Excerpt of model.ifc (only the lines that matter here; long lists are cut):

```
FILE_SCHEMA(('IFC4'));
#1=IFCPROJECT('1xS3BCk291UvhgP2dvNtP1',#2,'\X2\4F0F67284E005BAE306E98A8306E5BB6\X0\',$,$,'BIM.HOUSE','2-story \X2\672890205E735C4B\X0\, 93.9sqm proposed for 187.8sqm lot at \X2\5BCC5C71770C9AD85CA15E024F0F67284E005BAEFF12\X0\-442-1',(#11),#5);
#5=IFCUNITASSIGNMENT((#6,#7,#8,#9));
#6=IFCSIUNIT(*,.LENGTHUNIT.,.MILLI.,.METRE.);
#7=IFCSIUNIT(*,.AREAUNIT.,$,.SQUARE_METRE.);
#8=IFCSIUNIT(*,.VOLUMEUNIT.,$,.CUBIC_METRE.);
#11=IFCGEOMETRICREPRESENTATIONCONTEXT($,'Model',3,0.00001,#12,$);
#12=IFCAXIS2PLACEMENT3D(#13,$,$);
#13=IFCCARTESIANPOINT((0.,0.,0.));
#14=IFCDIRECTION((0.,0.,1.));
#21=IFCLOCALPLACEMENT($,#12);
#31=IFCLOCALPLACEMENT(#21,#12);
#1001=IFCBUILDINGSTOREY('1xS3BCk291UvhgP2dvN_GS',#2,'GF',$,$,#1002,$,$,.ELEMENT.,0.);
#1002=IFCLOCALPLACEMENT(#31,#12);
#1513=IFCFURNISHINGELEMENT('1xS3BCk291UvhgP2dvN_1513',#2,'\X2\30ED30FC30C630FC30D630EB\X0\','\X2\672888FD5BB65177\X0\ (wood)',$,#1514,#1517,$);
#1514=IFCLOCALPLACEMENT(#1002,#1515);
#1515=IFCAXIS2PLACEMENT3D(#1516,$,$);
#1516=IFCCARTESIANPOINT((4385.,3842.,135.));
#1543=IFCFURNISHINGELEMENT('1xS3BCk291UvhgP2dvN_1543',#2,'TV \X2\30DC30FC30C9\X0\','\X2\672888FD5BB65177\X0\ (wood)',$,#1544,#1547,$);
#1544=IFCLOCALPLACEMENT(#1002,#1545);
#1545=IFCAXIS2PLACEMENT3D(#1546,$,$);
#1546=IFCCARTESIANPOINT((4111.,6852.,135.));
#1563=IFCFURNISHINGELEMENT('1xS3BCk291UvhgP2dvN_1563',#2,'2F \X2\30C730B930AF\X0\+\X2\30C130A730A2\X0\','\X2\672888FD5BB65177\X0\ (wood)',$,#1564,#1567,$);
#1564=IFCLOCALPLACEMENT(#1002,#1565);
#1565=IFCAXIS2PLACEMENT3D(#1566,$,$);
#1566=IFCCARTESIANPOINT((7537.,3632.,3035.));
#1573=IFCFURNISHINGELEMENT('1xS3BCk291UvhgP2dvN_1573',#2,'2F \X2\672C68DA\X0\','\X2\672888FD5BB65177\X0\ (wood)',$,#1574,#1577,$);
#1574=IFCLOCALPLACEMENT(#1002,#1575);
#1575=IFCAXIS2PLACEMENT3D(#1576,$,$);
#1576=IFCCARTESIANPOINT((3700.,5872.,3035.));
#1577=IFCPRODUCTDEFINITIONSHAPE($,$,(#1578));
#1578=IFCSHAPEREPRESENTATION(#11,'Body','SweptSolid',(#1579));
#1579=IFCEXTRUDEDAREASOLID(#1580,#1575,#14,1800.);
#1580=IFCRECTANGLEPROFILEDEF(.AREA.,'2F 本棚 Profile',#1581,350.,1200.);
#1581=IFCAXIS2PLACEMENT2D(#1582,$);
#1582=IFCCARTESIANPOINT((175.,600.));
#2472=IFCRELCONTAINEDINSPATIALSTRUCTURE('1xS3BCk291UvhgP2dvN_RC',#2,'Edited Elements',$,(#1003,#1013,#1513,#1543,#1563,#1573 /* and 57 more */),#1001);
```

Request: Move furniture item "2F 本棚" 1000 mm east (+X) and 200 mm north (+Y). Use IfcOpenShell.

```python
import ifcopenshell
import ifcopenshell.api.geometry
import ifcopenshell.util.placement
import ifcopenshell.util.unit

model = ifcopenshell.open("model.ifc")
unit_scale = ifcopenshell.util.unit.calculate_unit_scale(model)

item = model.by_guid("1xS3BCk291UvhgP2dvN_1573")
matrix = ifcopenshell.util.placement.get_local_placement(item.ObjectPlacement)
matrix[0, 3] += 1 / unit_scale
matrix[1, 3] += 0.2 / unit_scale
ifcopenshell.api.geometry.edit_object_placement(model, product=item, matrix=matrix, is_si=False)

print(ifcopenshell.util.placement.get_local_placement(item.ObjectPlacement).round(3) + 0.0)

model.write("model_rev.ifc")
```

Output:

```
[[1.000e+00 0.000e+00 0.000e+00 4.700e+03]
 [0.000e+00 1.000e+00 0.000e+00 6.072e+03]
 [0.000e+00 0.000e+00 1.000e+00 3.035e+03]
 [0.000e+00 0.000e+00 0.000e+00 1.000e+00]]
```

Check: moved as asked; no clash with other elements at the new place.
